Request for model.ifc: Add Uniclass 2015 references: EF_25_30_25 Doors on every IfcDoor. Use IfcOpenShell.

First a look at what the model holds.

```python
import ifcopenshell

model = ifcopenshell.open("model.ifc")
print(model.schema)
print("classifications:", [c.Name for c in model.by_type("IfcClassification")])
for ifc_class in ("IfcDoor", "IfcRoof", "IfcStair", "IfcWall", "IfcWindow"):
    print(ifc_class, len(model.by_type(ifc_class)))
```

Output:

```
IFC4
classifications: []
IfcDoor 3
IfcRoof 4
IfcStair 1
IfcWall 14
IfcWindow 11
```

```python
import ifcopenshell
import ifcopenshell.api.classification

model = ifcopenshell.open("model.ifc")

system = ifcopenshell.api.classification.add_classification(model, classification="Uniclass 2015")

codes = {
    "IfcDoor": ("EF_25_30_25", "Doors"),
}
for ifc_class, (code, name) in codes.items():
    products = model.by_type(ifc_class)
    ifcopenshell.api.classification.add_reference(
        model, products=products, classification=system, identification=code, name=name
    )
    print(code, len(products))

model.write("model-out.ifc")
```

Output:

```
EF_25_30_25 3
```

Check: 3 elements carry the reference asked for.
